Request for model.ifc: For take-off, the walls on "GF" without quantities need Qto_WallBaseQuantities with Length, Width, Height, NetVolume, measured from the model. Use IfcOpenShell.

First a look at what the model holds.

```python
import ifcopenshell
import ifcopenshell.util.element
import ifcopenshell.util.unit

model = ifcopenshell.open("model.ifc")
print(model.schema)
for unit_type in ("LENGTHUNIT", "AREAUNIT", "VOLUMEUNIT"):
    print(unit_type, ifcopenshell.util.unit.calculate_unit_scale(model, unit_type))
storey = next(s for s in model.by_type("IfcBuildingStorey") if s.Name == "GF")
walls = [e for e in ifcopenshell.util.element.get_decomposition(storey) if e.is_a("IfcWall")]
for e in sorted(walls, key=lambda e: e.id()):
    print(e.id(), e.is_a(), e.Name, list(ifcopenshell.util.element.get_psets(e, qtos_only=True)), sep=" | ")
```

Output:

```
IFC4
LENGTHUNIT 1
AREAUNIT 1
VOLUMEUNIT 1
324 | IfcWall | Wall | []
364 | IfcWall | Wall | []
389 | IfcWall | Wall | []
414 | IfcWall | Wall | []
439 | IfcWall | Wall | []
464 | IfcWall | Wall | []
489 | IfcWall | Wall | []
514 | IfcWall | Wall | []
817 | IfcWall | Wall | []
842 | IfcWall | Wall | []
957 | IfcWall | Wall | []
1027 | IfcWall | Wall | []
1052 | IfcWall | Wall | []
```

```python
import ifcopenshell
import ifcopenshell.api.pset
import ifcopenshell.geom
import ifcopenshell.util.element
import ifcopenshell.util.shape
import ifcopenshell.util.unit

model = ifcopenshell.open("model.ifc")
unit_scale = ifcopenshell.util.unit.calculate_unit_scale(model)
volume_scale = ifcopenshell.util.unit.calculate_unit_scale(model, "VOLUMEUNIT")
settings = ifcopenshell.geom.settings()

storey = next(s for s in model.by_type("IfcBuildingStorey") if s.Name == "GF")
walls = [e for e in ifcopenshell.util.element.get_decomposition(storey) if e.is_a("IfcWall")]

for e in sorted(walls, key=lambda e: e.id()):
    if ifcopenshell.util.element.get_psets(e, qtos_only=True, should_inherit=False):
        continue
    # Geometry comes back in metres, in the element's own axes.
    shape = ifcopenshell.geom.create_shape(settings, e)
    values = {
        "Length": ifcopenshell.util.shape.get_x(shape.geometry) / unit_scale,
        "Width": ifcopenshell.util.shape.get_y(shape.geometry) / unit_scale,
        "Height": ifcopenshell.util.shape.get_z(shape.geometry) / unit_scale,
        "NetVolume": ifcopenshell.util.shape.get_volume(shape.geometry) / volume_scale,
    }
    qto = ifcopenshell.api.pset.add_qto(model, product=e, name="Qto_WallBaseQuantities")
    ifcopenshell.api.pset.edit_qto(model, qto=qto, properties=values)
    print(e.id(), {k: round(v, 3) for k, v in values.items()})

model.write("model_edited.ifc")
```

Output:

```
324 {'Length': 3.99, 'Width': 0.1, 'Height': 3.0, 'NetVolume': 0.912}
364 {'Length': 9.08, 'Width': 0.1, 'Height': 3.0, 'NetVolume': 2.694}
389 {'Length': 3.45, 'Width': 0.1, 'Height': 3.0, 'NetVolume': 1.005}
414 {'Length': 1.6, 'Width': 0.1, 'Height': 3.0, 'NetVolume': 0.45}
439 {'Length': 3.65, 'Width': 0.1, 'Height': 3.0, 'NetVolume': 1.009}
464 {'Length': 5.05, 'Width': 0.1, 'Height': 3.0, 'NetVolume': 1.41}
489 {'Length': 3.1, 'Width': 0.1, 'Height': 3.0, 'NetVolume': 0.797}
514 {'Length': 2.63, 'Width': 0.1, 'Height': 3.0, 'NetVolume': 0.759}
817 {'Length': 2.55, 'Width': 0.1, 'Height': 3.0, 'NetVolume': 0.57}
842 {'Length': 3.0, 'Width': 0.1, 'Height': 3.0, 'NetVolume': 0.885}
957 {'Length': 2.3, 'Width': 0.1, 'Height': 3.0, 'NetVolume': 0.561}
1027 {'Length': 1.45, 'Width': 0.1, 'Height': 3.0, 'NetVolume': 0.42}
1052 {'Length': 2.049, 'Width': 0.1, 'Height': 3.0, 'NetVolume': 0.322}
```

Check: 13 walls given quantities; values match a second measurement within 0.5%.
